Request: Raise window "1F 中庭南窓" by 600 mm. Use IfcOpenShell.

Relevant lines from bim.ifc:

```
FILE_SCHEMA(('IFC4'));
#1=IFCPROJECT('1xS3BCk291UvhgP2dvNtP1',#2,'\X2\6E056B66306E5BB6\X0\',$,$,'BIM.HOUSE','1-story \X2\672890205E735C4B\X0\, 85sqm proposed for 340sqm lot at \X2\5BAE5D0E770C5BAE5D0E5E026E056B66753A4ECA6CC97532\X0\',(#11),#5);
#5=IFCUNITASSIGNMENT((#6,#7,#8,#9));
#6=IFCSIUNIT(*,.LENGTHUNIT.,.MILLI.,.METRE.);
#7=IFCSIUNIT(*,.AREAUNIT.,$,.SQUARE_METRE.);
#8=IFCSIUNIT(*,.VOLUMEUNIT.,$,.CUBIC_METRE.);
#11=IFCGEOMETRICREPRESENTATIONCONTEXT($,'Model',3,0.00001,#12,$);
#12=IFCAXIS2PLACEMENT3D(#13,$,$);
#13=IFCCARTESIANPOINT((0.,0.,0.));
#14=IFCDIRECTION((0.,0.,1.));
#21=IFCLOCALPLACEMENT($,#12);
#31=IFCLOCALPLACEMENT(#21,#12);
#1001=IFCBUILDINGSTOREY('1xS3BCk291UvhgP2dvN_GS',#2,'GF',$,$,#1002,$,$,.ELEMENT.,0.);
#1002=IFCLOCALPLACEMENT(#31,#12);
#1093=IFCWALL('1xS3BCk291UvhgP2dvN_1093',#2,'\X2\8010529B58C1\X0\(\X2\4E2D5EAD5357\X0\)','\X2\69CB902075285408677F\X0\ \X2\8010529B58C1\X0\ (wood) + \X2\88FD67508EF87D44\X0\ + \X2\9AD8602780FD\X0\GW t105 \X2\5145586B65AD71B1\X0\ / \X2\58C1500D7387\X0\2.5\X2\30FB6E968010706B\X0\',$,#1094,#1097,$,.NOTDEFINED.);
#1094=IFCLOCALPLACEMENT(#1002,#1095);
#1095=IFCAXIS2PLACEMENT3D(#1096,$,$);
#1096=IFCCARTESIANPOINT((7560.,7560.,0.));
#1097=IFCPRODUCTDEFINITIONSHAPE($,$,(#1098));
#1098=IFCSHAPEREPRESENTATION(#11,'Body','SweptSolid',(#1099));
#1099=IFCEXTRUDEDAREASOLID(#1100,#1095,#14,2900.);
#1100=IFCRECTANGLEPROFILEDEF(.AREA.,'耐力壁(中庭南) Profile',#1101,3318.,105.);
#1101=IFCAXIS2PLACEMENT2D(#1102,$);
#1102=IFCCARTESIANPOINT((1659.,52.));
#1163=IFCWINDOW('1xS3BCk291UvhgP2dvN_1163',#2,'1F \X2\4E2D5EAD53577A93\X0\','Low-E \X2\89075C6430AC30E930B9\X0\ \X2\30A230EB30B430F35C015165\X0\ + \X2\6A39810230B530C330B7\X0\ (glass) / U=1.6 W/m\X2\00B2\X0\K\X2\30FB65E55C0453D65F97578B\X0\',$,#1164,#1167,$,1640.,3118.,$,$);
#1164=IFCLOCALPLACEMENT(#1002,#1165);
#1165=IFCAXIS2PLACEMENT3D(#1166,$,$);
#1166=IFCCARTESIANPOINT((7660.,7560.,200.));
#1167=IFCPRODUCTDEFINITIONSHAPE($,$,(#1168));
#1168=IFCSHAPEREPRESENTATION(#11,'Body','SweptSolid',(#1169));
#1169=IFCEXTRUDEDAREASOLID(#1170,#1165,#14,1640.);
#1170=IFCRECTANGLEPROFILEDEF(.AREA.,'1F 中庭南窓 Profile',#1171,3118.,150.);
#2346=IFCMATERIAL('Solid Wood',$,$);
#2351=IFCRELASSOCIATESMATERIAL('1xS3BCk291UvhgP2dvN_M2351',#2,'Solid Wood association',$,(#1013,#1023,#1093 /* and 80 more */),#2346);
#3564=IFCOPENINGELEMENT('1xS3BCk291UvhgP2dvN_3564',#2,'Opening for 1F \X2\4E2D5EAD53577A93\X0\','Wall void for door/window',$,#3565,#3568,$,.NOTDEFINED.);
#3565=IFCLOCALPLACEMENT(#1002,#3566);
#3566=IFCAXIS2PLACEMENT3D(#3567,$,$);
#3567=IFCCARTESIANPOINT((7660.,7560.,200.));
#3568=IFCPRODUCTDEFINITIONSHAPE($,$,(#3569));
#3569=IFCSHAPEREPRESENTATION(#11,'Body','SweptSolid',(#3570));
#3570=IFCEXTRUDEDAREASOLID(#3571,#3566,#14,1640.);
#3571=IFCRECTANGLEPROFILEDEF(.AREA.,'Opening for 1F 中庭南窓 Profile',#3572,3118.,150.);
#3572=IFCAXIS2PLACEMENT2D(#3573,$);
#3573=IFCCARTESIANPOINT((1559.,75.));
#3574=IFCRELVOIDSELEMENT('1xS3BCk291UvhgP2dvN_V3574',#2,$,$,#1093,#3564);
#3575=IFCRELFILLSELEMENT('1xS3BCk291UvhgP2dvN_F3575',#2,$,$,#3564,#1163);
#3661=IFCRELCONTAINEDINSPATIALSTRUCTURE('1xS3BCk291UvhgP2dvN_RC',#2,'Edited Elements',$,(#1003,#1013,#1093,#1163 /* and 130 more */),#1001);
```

```python
import numpy as np
import ifcopenshell
import ifcopenshell.api.geometry
import ifcopenshell.util.placement
import ifcopenshell.util.unit

model = ifcopenshell.open("bim.ifc")
unit_scale = ifcopenshell.util.unit.calculate_unit_scale(model)

window = model.by_id(1163)
opening = window.FillsVoids[0].RelatingOpeningElement
dz = 600.0

shift = np.array([0.0, 0.0, dz])
# The window is not placed relative to its opening, so move both.
for product in (opening, window):
    matrix = ifcopenshell.util.placement.get_local_placement(product.ObjectPlacement)
    matrix[:3, 3] += shift
    ifcopenshell.api.geometry.edit_object_placement(model, product=product, matrix=matrix, is_si=False)

print(f"moved by {dz * unit_scale:+.3f} m")

model.write("bim_rev.ifc")
```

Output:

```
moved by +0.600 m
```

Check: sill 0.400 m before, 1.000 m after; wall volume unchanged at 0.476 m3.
